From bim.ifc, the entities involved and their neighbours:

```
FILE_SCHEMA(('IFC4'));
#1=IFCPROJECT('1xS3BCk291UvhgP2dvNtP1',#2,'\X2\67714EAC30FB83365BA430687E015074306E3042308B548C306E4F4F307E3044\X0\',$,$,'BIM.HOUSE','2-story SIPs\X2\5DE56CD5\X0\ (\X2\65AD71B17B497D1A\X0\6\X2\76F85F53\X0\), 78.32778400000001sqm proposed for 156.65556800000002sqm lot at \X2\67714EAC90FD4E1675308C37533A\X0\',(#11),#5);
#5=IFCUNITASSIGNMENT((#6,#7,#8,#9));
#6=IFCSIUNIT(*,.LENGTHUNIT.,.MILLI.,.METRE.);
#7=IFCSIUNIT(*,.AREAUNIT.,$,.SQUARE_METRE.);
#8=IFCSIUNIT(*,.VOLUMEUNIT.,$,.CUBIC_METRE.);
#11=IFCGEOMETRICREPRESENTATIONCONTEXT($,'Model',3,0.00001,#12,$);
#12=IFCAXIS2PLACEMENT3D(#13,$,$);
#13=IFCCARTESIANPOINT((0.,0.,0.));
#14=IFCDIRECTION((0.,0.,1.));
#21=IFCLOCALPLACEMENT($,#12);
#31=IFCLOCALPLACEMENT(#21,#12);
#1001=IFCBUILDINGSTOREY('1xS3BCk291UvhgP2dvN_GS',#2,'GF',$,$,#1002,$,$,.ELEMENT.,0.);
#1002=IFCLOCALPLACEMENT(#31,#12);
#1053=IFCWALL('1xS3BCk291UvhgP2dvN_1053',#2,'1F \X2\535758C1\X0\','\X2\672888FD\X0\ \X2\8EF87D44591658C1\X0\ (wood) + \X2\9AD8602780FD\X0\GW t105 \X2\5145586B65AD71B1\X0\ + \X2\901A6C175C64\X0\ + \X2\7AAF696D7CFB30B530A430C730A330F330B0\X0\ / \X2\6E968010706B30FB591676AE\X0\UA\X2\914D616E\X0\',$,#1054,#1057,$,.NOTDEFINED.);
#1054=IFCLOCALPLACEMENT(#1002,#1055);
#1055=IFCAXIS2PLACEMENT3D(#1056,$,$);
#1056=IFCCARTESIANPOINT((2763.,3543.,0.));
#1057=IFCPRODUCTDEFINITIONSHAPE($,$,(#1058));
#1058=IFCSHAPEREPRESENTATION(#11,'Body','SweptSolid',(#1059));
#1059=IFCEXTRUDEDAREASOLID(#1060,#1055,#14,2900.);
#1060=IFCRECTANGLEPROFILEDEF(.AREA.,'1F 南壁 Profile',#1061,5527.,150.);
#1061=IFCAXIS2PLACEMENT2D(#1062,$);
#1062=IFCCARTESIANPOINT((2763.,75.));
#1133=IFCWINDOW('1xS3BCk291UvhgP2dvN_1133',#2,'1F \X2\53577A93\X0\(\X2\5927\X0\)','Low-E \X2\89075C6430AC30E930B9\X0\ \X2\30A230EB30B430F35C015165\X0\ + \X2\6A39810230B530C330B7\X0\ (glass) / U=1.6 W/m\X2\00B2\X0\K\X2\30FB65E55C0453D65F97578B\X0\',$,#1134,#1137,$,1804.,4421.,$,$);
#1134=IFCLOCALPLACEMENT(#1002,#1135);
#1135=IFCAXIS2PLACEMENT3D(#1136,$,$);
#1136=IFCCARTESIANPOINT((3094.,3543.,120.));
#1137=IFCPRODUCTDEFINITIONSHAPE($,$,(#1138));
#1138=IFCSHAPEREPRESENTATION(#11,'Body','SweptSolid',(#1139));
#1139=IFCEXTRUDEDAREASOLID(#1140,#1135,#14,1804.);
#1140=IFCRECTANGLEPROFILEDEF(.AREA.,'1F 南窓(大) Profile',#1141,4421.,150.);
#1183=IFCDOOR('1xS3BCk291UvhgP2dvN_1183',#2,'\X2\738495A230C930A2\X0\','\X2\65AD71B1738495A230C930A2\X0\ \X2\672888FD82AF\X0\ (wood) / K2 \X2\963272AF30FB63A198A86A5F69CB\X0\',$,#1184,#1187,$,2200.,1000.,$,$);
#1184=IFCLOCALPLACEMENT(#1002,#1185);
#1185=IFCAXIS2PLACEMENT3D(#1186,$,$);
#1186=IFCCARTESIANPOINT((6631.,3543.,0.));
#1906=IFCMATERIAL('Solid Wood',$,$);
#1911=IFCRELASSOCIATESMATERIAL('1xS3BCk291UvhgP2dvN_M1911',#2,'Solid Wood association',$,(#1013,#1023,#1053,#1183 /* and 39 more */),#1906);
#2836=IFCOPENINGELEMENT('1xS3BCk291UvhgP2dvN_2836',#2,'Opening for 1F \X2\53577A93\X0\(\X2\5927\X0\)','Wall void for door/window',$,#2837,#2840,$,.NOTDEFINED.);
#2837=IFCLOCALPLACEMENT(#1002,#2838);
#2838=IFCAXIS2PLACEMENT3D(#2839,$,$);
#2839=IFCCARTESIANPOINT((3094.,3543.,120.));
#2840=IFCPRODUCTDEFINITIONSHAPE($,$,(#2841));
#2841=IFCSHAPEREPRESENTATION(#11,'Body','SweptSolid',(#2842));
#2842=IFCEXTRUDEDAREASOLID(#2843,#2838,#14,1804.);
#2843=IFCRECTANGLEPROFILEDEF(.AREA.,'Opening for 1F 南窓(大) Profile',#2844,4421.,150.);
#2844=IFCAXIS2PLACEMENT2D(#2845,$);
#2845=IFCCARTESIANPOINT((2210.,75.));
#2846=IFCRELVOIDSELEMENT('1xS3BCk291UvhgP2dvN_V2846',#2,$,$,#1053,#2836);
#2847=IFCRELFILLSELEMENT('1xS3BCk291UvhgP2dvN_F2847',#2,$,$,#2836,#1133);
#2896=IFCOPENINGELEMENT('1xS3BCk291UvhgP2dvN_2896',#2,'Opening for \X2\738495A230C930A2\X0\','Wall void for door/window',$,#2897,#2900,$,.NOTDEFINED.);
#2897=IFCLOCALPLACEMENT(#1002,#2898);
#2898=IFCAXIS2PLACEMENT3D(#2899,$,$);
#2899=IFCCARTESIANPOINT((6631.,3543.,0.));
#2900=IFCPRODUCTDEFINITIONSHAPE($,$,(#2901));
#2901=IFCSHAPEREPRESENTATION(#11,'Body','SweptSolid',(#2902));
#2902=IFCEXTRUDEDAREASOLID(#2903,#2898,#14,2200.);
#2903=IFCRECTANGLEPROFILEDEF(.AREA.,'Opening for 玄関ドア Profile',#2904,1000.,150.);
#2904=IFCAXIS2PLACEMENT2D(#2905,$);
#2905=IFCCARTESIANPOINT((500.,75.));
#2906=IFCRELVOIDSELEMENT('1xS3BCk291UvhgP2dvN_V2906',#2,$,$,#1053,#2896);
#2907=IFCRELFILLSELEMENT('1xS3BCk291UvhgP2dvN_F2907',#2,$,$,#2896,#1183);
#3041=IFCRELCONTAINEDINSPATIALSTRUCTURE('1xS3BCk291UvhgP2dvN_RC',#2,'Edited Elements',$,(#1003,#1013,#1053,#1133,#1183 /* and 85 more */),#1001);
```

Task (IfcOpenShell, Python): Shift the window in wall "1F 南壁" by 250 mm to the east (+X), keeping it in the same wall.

```python
import ifcopenshell
import ifcopenshell.api.geometry
import ifcopenshell.util.placement
import ifcopenshell.util.unit

model = ifcopenshell.open("bim.ifc")
unit_scale = ifcopenshell.util.unit.calculate_unit_scale(model)

window = model.by_guid("1xS3BCk291UvhgP2dvN_1133")
opening = window.FillsVoids[0].RelatingOpeningElement
wall = opening.VoidsElements[0].RelatingBuildingElement

wall_matrix = ifcopenshell.util.placement.get_local_placement(wall.ObjectPlacement)
shift = wall_matrix[:3, 0] * 0.25 / unit_scale
before = ifcopenshell.util.placement.get_local_placement(window.ObjectPlacement)[:3, 3].copy()

# The window is not placed relative to its opening, so move both.
for product in (opening, window):
    matrix = ifcopenshell.util.placement.get_local_placement(product.ObjectPlacement)
    matrix[:3, 3] += shift
    ifcopenshell.api.geometry.edit_object_placement(model, product=product, matrix=matrix, is_si=False)

after = ifcopenshell.util.placement.get_local_placement(window.ObjectPlacement)[:3, 3]
print("window moved by", (after - before).round(3) + 0.0)

model.write("bim_v2.ifc")
```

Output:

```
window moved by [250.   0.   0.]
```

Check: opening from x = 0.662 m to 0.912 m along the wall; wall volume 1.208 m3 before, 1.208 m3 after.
